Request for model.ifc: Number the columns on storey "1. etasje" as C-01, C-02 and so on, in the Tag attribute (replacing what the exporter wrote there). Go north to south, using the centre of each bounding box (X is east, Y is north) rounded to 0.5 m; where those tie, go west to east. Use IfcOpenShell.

First a look at what the model holds.

```python
import ifcopenshell
import ifcopenshell.util.element
import ifcopenshell.util.placement

model = ifcopenshell.open("model.ifc")
print(model.schema)
storey = next(s for s in model.by_type("IfcBuildingStorey") if s.Name == "1. etasje")
columns = [e for e in ifcopenshell.util.element.get_decomposition(storey) if e.is_a("IfcColumn")]
for e in sorted(columns, key=lambda e: e.id()):
    origin = ifcopenshell.util.placement.get_local_placement(e.ObjectPlacement)[:3, 3]
    print(e.id(), e.Tag, e.Name, origin.round(2) + 0.0, sep=" | ")
```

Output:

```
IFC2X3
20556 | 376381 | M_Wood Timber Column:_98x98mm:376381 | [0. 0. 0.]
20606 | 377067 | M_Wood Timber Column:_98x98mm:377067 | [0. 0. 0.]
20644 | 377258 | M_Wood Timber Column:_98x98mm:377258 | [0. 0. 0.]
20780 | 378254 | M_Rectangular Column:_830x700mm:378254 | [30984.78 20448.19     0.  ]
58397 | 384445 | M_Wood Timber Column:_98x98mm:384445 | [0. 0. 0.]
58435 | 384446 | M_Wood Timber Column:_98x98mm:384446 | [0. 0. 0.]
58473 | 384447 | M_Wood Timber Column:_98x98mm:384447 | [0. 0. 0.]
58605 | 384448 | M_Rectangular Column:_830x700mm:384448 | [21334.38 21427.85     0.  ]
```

```python
import ifcopenshell
import ifcopenshell.geom
import ifcopenshell.util.element
import ifcopenshell.util.shape

model = ifcopenshell.open("model.ifc")
settings = ifcopenshell.geom.settings()
settings.set("use-world-coords", True)


def centre(element):
    shape = ifcopenshell.geom.create_shape(settings, element)
    return ifcopenshell.util.shape.get_bbox_centroid(shape.geometry)


storey = next(s for s in model.by_type("IfcBuildingStorey") if s.Name == "1. etasje")
columns = [e for e in ifcopenshell.util.element.get_decomposition(storey) if e.is_a("IfcColumn")]

# Insertion points can sit at a corner or the storey origin, so sort by the geometry (in metres).
centres = {e: centre(e) for e in columns}
columns.sort(key=lambda e: (-round(centres[e][1] / 0.5), centres[e][0]))

for i, e in enumerate(columns, start=1):
    number = f"C-{i:02d}"
    e.Tag = number
    print(e.id(), number)

model.write("model_edited.ifc")
```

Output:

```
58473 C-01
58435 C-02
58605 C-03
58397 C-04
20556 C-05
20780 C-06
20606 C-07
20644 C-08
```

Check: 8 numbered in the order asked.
